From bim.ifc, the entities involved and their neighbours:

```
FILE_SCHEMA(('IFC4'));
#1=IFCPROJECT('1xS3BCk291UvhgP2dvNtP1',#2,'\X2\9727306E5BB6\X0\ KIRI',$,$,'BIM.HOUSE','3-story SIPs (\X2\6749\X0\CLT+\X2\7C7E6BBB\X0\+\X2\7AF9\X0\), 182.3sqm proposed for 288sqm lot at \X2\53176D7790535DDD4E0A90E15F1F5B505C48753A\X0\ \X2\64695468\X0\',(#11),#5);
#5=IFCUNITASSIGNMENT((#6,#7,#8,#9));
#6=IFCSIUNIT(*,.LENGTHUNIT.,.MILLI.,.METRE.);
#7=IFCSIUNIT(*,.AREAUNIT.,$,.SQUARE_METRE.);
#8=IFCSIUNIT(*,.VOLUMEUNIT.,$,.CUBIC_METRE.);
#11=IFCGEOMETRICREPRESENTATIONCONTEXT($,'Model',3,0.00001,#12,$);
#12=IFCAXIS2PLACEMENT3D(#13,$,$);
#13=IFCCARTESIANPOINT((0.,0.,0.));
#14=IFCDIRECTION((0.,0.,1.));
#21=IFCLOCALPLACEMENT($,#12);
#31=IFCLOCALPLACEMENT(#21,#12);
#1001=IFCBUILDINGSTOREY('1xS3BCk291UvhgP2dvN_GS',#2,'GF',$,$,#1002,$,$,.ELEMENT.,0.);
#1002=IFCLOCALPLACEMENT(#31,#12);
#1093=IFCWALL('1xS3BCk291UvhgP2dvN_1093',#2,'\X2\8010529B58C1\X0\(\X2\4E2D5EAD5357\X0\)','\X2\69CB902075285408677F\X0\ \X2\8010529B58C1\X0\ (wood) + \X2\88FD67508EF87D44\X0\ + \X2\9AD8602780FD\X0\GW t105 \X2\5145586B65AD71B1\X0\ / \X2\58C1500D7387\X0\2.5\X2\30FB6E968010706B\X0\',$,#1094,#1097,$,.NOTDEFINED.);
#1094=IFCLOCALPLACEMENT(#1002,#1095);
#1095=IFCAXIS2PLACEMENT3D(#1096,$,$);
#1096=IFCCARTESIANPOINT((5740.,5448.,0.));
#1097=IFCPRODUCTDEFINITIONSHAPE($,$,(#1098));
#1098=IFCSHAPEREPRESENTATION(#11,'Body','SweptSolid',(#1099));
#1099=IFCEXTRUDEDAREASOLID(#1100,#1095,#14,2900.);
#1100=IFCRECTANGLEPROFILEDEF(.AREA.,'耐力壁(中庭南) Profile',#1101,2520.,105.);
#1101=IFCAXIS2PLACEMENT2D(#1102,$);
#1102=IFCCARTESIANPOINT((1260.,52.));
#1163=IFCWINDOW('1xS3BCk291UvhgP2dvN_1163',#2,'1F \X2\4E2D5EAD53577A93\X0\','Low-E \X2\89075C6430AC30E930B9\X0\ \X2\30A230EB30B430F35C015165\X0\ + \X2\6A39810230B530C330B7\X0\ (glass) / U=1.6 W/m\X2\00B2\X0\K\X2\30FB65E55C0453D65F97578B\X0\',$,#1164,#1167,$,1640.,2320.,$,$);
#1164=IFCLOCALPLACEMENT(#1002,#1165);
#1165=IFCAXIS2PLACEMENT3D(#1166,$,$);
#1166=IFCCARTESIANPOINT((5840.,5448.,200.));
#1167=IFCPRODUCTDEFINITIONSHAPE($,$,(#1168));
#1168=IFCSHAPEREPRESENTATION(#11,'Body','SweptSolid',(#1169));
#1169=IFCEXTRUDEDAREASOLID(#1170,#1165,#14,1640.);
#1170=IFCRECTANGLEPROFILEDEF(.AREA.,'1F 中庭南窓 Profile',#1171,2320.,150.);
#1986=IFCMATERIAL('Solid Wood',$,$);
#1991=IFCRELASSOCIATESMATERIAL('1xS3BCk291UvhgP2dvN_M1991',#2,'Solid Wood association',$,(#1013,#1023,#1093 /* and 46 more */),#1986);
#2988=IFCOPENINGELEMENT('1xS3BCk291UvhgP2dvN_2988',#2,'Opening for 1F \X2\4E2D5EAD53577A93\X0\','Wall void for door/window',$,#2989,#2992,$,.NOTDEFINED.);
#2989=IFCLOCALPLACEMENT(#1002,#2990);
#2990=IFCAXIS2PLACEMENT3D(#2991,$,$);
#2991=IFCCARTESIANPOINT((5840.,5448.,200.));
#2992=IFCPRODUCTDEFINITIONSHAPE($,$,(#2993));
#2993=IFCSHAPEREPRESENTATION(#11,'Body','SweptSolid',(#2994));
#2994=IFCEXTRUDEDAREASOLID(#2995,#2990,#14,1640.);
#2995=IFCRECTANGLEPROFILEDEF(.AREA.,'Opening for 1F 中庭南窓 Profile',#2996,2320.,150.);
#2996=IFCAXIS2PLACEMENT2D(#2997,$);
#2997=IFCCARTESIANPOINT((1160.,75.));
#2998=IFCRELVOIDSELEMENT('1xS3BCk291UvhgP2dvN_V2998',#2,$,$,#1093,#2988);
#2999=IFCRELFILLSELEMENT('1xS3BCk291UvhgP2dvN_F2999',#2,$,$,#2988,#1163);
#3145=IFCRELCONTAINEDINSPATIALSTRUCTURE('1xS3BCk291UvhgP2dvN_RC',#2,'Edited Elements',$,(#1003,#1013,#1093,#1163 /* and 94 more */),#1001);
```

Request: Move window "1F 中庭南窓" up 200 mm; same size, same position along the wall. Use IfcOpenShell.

```python
import numpy as np
import ifcopenshell
import ifcopenshell.api.geometry
import ifcopenshell.util.placement
import ifcopenshell.util.unit

model = ifcopenshell.open("bim.ifc")
unit_scale = ifcopenshell.util.unit.calculate_unit_scale(model)

window = model.by_guid("1xS3BCk291UvhgP2dvN_1163")
opening = window.FillsVoids[0].RelatingOpeningElement
dz = 200.0

shift = np.array([0.0, 0.0, dz])
# The window is not placed relative to its opening, so move both.
for product in (opening, window):
    matrix = ifcopenshell.util.placement.get_local_placement(product.ObjectPlacement)
    matrix[:3, 3] += shift
    ifcopenshell.api.geometry.edit_object_placement(model, product=product, matrix=matrix, is_si=False)

print(f"moved by {dz * unit_scale:+.3f} m")

model.write("bim_edited.ifc")
```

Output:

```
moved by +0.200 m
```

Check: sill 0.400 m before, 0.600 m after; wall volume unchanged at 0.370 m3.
